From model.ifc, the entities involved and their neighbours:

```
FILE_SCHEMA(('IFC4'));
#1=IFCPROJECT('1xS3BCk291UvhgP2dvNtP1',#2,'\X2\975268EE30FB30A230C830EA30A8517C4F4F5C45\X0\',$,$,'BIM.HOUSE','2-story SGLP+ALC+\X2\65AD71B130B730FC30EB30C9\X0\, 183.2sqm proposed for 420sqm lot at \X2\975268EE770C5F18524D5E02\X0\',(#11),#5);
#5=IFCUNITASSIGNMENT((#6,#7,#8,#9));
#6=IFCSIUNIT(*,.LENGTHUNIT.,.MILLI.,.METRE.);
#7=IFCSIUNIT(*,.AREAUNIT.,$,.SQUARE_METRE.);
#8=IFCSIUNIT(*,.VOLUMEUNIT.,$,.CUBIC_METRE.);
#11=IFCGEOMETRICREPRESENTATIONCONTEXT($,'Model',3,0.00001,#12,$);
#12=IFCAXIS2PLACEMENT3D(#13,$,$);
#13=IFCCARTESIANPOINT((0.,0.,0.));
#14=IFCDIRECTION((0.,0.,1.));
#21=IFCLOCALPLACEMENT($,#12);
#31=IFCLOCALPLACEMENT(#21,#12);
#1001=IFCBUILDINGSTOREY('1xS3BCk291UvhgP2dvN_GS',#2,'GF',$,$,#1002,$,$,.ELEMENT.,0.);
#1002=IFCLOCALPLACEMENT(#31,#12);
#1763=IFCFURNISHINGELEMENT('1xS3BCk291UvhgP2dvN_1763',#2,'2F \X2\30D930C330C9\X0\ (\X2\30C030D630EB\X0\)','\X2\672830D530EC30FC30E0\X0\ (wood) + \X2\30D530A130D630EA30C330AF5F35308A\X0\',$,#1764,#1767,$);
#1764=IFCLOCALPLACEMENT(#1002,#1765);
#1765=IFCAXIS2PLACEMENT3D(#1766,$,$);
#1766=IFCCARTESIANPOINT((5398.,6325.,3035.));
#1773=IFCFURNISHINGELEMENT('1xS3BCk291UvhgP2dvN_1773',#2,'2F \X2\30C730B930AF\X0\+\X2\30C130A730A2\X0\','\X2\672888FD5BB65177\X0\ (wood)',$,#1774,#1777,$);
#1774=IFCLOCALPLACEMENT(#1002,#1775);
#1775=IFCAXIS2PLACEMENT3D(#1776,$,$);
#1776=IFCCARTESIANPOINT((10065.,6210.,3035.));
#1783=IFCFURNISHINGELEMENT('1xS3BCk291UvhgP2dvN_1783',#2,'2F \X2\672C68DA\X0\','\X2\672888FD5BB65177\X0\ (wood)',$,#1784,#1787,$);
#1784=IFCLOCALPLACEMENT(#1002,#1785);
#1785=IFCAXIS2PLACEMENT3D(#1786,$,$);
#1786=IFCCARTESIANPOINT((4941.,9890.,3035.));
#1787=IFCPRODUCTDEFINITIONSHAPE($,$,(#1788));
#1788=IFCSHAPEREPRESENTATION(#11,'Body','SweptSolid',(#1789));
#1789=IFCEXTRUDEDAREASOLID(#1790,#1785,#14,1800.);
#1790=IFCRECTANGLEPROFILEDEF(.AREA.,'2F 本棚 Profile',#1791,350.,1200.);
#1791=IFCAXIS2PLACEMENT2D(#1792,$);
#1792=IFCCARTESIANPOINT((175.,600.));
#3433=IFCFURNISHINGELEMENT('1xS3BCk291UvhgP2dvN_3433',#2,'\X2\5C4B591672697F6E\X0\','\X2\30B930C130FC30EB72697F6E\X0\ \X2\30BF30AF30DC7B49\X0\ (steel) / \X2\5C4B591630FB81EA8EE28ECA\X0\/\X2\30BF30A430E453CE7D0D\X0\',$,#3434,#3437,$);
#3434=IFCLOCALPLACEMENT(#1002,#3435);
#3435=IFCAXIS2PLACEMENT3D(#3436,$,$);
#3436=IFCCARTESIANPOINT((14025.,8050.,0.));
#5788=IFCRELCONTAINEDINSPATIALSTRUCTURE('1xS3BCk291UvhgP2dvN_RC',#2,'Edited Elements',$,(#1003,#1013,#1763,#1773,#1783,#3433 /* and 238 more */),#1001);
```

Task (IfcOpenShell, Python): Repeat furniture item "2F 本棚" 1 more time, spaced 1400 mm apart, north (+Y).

```python
import numpy as np
import ifcopenshell
import ifcopenshell.api.geometry
import ifcopenshell.api.root
import ifcopenshell.util.element
import ifcopenshell.util.placement
import ifcopenshell.util.unit

model = ifcopenshell.open("model.ifc")
unit_scale = ifcopenshell.util.unit.calculate_unit_scale(model)


def reuse_history(source, copy):
    """copy_class also copies each property set's owner history, people and application; keep the originals."""
    for rel in copy.IsDefinedBy:
        if rel.is_a("IfcRelDefinesByProperties") and (history := rel.RelatingPropertyDefinition.OwnerHistory):
            rel.RelatingPropertyDefinition.OwnerHistory = source.OwnerHistory
            ifcopenshell.util.element.remove_deep2(model, history)


source = model.by_guid("1xS3BCk291UvhgP2dvN_1783")
base = ifcopenshell.util.placement.get_local_placement(source.ObjectPlacement)
step = np.array([0.0, 1.0, 0.0]) * 1.4 / unit_scale

for i in range(1, 2):
    copy = ifcopenshell.api.root.copy_class(model, product=source)
    copy.Representation = ifcopenshell.util.element.copy_deep(
        model, source.Representation, exclude=["IfcGeometricRepresentationContext", "IfcRepresentationMap"]
    )
    reuse_history(source, copy)
    matrix = base.copy()
    matrix[:3, 3] += i * step
    print("added at", matrix[:3, 3].round(3) + 0.0)
    ifcopenshell.api.geometry.edit_object_placement(model, product=copy, matrix=matrix, is_si=False)

model.write("model-out.ifc")
```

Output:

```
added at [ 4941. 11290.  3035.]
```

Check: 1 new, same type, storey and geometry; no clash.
